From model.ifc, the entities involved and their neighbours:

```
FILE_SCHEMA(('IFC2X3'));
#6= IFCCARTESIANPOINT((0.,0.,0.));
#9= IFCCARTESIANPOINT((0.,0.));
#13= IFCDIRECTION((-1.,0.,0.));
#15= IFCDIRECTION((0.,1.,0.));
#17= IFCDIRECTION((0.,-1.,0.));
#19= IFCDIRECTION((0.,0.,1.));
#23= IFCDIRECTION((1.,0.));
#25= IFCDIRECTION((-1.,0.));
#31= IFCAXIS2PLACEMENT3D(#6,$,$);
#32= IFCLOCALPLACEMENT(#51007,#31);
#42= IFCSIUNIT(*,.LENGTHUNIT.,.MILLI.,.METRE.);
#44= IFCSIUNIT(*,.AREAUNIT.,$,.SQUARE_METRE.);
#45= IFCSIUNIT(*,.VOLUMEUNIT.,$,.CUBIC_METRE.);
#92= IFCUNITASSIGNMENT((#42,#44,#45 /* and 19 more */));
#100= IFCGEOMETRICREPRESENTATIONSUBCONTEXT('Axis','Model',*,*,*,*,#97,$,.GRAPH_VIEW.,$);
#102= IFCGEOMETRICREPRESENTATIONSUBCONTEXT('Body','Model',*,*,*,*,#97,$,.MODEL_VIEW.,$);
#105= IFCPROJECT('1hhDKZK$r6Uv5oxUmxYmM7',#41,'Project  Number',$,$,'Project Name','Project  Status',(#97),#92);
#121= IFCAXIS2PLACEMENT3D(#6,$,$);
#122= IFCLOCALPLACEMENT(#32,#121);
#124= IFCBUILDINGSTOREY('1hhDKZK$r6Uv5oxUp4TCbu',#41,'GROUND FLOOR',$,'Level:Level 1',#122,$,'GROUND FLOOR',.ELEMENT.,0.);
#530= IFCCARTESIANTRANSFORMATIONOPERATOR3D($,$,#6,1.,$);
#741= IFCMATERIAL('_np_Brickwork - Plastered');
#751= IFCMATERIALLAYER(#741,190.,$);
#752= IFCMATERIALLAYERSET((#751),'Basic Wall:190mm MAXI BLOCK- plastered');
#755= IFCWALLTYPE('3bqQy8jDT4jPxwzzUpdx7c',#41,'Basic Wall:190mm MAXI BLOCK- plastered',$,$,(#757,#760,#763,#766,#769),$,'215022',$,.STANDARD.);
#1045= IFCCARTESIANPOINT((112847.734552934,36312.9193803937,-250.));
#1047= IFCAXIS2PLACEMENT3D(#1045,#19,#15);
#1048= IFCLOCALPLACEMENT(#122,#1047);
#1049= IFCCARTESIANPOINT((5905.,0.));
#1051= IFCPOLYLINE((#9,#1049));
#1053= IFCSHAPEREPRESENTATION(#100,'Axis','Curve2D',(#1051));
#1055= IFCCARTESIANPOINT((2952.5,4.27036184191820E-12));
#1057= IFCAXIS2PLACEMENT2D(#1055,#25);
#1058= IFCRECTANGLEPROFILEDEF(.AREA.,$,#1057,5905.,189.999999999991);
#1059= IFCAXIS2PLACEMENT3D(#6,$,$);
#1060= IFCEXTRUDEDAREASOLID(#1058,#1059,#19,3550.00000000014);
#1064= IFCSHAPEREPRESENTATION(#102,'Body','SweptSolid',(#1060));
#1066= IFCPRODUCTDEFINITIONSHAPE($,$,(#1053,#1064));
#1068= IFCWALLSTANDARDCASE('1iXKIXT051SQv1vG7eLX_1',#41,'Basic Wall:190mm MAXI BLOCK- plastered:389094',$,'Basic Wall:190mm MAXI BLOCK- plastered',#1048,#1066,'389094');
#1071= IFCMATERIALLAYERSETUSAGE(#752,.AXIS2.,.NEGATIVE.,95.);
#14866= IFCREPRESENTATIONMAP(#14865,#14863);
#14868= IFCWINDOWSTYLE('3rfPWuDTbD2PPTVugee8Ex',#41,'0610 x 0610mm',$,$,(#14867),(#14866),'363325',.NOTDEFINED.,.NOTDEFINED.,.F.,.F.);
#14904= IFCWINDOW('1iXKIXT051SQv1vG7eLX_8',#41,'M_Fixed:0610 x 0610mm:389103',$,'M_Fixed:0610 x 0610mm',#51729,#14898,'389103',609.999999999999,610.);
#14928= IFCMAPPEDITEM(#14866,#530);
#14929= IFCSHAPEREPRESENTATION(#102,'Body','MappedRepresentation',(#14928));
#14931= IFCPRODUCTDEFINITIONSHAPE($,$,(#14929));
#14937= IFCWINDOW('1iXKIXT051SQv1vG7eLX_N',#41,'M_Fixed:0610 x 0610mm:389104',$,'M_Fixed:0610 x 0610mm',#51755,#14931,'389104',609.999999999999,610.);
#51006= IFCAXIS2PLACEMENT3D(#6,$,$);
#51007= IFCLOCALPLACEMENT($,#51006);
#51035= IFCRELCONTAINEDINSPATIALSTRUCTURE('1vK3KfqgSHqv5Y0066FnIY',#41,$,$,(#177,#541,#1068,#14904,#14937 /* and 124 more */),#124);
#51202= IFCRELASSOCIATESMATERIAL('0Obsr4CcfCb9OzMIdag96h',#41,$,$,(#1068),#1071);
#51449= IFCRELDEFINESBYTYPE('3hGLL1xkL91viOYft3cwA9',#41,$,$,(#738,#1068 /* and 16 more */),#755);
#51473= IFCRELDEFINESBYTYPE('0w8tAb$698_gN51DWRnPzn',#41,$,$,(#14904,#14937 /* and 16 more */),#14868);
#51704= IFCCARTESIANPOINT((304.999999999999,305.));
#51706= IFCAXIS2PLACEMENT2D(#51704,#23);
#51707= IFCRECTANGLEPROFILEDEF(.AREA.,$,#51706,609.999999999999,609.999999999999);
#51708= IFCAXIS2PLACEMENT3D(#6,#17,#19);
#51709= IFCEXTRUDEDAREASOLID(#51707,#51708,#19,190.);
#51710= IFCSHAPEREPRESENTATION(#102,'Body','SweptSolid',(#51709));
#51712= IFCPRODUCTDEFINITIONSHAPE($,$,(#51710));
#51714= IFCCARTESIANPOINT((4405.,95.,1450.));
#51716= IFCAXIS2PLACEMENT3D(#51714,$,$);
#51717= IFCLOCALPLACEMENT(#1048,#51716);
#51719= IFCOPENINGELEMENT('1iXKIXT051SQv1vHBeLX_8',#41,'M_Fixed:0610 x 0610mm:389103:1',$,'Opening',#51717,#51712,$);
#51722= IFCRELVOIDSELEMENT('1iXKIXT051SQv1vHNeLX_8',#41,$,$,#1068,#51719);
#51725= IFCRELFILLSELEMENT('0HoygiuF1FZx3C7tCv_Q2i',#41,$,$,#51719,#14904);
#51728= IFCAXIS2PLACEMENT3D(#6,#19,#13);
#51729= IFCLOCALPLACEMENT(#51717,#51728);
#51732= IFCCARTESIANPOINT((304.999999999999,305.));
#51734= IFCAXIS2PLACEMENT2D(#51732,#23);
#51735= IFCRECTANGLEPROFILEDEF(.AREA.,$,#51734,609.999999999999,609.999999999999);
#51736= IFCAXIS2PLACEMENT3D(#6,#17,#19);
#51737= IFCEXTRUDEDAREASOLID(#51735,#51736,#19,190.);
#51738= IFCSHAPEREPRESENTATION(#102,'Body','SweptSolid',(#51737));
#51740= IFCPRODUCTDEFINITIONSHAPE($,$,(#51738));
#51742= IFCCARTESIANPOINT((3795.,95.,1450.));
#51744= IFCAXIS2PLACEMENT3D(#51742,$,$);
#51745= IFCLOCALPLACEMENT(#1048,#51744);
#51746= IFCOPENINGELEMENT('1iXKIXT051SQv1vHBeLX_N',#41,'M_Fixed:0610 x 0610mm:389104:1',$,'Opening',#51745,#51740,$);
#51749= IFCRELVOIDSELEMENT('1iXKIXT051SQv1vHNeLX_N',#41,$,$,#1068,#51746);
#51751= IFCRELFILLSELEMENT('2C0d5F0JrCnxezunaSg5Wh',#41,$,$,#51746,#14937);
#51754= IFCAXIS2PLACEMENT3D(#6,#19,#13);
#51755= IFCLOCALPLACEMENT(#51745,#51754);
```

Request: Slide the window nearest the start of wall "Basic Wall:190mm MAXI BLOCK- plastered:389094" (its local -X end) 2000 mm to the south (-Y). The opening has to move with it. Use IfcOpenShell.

```python
import ifcopenshell
import ifcopenshell.api.geometry
import ifcopenshell.util.placement
import ifcopenshell.util.unit

model = ifcopenshell.open("model.ifc")
unit_scale = ifcopenshell.util.unit.calculate_unit_scale(model)

window = model.by_guid("1iXKIXT051SQv1vG7eLX_N")
opening = window.FillsVoids[0].RelatingOpeningElement
wall = opening.VoidsElements[0].RelatingBuildingElement

wall_matrix = ifcopenshell.util.placement.get_local_placement(wall.ObjectPlacement)
shift = wall_matrix[:3, 0] * -2 / unit_scale
before = ifcopenshell.util.placement.get_local_placement(window.ObjectPlacement)[:3, 3].copy()

# The window is placed relative to its opening, so it follows when the opening moves.
matrix = ifcopenshell.util.placement.get_local_placement(opening.ObjectPlacement)
matrix[:3, 3] += shift
ifcopenshell.api.geometry.edit_object_placement(
    model, product=opening, matrix=matrix, is_si=False, should_transform_children=True
)

after = ifcopenshell.util.placement.get_local_placement(window.ObjectPlacement)[:3, 3]
print("window moved by", (after - before).round(3) + 0.0)

model.write("model-out.ifc")
```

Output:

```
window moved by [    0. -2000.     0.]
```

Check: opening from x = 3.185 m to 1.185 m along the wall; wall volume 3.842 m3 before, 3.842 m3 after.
